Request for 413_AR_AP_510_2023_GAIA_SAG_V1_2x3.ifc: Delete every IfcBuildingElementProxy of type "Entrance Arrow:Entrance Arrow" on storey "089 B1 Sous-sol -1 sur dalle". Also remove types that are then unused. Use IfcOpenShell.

First a look at what the model holds.

```python
import ifcopenshell
import ifcopenshell.util.element

model = ifcopenshell.open("413_AR_AP_510_2023_GAIA_SAG_V1_2x3.ifc")
print(model.schema)
storey = next(s for s in model.by_type("IfcBuildingStorey") if s.Name == "089 B1 Sous-sol -1 sur dalle")
proxies = [e for e in ifcopenshell.util.element.get_decomposition(storey) if e.is_a("IfcBuildingElementProxy")]
seen = {}
for e in proxies:
    element_type = ifcopenshell.util.element.get_type(e)
    name = element_type.Name if element_type not in (None, e) else None
    seen[name] = seen.get(name, 0) + 1
for name, count in sorted(seen.items(), key=str):
    print(count, "x", name)
```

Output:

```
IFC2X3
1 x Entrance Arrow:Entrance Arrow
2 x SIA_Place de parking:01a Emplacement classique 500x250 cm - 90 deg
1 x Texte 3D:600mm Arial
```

```python
import ifcopenshell
import ifcopenshell.api.root
import ifcopenshell.util.element

model = ifcopenshell.open("413_AR_AP_510_2023_GAIA_SAG_V1_2x3.ifc")

storey = next(s for s in model.by_type("IfcBuildingStorey") if s.Name == "089 B1 Sous-sol -1 sur dalle")
proxies = [e for e in ifcopenshell.util.element.get_decomposition(storey) if e.is_a("IfcBuildingElementProxy")]
targets = [e for e in proxies if (t := ifcopenshell.util.element.get_type(e)) not in (None, e) and t.Name == "Entrance Arrow:Entrance Arrow"]
types = {ifcopenshell.util.element.get_type(e) for e in targets} - {None, *targets}

for e in targets:
    ifcopenshell.api.root.remove_product(model, product=e)
print(len(targets), "removed")

unused = [t for t in types if not ifcopenshell.util.element.get_types(t)]
for t in unused:
    ifcopenshell.api.root.remove_product(model, product=t)
print(len(unused), "unused types removed")

model.write("413_AR_AP_510_2023_GAIA_SAG_V1_2x3-out.ifc")
```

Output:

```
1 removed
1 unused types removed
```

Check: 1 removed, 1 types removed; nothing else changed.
